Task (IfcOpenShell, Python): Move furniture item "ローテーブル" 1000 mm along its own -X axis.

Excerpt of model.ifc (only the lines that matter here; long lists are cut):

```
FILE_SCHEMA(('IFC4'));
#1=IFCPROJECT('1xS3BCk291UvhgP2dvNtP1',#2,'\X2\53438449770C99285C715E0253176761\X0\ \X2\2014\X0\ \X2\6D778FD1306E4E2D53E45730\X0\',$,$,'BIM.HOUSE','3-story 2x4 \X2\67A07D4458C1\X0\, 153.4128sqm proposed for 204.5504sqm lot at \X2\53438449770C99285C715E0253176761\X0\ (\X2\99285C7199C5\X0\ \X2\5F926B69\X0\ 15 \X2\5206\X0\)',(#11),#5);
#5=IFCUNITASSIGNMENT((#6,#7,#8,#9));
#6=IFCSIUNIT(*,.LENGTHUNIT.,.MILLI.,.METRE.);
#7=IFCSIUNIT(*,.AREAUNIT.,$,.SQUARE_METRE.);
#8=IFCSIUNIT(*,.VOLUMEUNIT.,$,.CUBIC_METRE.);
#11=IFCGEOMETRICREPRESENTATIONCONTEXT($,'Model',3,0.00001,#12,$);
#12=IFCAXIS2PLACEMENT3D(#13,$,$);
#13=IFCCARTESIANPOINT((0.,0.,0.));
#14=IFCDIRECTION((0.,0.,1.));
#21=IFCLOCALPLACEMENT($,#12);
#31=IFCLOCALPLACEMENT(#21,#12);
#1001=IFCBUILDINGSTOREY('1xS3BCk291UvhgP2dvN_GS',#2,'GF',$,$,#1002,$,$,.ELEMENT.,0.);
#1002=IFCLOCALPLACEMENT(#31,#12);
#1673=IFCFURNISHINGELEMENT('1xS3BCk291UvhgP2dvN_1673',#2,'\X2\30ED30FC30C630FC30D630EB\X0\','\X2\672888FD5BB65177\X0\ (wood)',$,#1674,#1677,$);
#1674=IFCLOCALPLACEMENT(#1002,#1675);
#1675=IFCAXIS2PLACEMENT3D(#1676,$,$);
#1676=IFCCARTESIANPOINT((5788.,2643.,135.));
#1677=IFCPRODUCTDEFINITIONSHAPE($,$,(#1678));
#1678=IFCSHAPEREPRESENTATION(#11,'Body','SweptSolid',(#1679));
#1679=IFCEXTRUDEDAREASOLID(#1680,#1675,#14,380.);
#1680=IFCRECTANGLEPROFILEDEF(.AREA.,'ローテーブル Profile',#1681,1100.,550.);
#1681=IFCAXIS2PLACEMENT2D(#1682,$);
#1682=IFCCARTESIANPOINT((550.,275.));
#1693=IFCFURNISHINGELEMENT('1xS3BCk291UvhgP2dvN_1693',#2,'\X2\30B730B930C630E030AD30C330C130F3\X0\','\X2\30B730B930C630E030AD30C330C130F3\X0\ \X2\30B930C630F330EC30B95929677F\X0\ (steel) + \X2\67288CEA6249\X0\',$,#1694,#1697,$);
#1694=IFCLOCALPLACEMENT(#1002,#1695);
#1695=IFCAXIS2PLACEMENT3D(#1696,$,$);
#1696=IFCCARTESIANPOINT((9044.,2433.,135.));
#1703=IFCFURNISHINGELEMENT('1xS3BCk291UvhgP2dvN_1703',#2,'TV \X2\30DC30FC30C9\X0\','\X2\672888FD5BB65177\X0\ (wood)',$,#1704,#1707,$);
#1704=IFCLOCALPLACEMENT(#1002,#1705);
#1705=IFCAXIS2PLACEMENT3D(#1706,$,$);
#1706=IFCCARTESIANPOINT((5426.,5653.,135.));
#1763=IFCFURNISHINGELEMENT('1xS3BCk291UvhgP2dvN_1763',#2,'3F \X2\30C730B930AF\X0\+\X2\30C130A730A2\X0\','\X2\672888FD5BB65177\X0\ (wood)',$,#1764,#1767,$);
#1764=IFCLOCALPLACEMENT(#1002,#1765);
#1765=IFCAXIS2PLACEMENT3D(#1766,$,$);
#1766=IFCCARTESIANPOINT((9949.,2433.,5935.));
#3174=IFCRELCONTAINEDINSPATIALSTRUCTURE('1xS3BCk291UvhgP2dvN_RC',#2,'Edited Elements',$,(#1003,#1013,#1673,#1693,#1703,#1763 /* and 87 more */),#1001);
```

```python
import ifcopenshell
import ifcopenshell.api.geometry
import ifcopenshell.util.placement
import ifcopenshell.util.unit

model = ifcopenshell.open("model.ifc")
unit_scale = ifcopenshell.util.unit.calculate_unit_scale(model)

item = model.by_guid("1xS3BCk291UvhgP2dvN_1673")
matrix = ifcopenshell.util.placement.get_local_placement(item.ObjectPlacement)
matrix[:3, 3] -= matrix[:3, 0] * 1 / unit_scale
ifcopenshell.api.geometry.edit_object_placement(model, product=item, matrix=matrix, is_si=False)

print(ifcopenshell.util.placement.get_local_placement(item.ObjectPlacement).round(3) + 0.0)

model.write("model_edited.ifc")
```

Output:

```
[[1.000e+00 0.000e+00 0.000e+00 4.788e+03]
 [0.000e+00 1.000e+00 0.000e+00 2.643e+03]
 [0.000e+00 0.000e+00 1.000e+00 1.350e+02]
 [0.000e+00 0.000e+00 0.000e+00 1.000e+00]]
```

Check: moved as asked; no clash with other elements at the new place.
